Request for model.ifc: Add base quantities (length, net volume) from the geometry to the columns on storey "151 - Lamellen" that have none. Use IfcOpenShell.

First a look at what the model holds.

```python
import ifcopenshell
import ifcopenshell.util.element
import ifcopenshell.util.unit

model = ifcopenshell.open("model.ifc")
print(model.schema)
for unit_type in ("LENGTHUNIT", "AREAUNIT", "VOLUMEUNIT"):
    print(unit_type, ifcopenshell.util.unit.calculate_unit_scale(model, unit_type))
storey = next(s for s in model.by_type("IfcBuildingStorey") if s.Name == "151 - Lamellen")
columns = [e for e in ifcopenshell.util.element.get_decomposition(storey) if e.is_a("IfcColumn")]
for e in sorted(columns, key=lambda e: e.id()):
    print(e.id(), e.is_a(), e.Name, list(ifcopenshell.util.element.get_psets(e, qtos_only=True)), sep=" | ")
```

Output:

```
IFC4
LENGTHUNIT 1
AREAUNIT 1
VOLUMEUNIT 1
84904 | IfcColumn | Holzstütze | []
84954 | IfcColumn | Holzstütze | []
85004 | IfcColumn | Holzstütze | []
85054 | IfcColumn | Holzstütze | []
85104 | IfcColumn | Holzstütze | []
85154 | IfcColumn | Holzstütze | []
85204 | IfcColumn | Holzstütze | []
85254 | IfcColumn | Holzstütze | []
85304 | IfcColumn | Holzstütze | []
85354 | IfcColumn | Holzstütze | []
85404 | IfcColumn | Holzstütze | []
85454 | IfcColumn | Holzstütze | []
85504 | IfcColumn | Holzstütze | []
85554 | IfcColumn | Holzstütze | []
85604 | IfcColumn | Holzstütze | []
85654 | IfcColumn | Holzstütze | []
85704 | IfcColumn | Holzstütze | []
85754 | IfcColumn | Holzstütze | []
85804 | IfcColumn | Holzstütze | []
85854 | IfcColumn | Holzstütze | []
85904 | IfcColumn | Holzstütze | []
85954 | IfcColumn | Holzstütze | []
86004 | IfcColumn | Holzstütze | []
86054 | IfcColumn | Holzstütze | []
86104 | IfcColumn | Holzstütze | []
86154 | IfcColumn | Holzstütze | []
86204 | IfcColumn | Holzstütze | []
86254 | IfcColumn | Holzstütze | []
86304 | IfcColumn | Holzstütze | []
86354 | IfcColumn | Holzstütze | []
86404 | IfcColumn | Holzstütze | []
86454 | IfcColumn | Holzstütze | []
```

```python
import ifcopenshell
import ifcopenshell.api.pset
import ifcopenshell.geom
import ifcopenshell.util.element
import ifcopenshell.util.shape
import ifcopenshell.util.unit

model = ifcopenshell.open("model.ifc")
unit_scale = ifcopenshell.util.unit.calculate_unit_scale(model)
volume_scale = ifcopenshell.util.unit.calculate_unit_scale(model, "VOLUMEUNIT")
settings = ifcopenshell.geom.settings()

storey = next(s for s in model.by_type("IfcBuildingStorey") if s.Name == "151 - Lamellen")
columns = [e for e in ifcopenshell.util.element.get_decomposition(storey) if e.is_a("IfcColumn")]

for e in sorted(columns, key=lambda e: e.id()):
    if ifcopenshell.util.element.get_psets(e, qtos_only=True, should_inherit=False):
        continue
    # Geometry comes back in metres, in the element's own axes.
    shape = ifcopenshell.geom.create_shape(settings, e)
    values = {
        "Length": ifcopenshell.util.shape.get_z(shape.geometry) / unit_scale,
        "NetVolume": ifcopenshell.util.shape.get_volume(shape.geometry) / volume_scale,
    }
    qto = ifcopenshell.api.pset.add_qto(model, product=e, name="Qto_ColumnBaseQuantities")
    ifcopenshell.api.pset.edit_qto(model, qto=qto, properties=values)
    print(e.id(), {k: round(v, 3) for k, v in values.items()})

model.write("model_updated.ifc")
```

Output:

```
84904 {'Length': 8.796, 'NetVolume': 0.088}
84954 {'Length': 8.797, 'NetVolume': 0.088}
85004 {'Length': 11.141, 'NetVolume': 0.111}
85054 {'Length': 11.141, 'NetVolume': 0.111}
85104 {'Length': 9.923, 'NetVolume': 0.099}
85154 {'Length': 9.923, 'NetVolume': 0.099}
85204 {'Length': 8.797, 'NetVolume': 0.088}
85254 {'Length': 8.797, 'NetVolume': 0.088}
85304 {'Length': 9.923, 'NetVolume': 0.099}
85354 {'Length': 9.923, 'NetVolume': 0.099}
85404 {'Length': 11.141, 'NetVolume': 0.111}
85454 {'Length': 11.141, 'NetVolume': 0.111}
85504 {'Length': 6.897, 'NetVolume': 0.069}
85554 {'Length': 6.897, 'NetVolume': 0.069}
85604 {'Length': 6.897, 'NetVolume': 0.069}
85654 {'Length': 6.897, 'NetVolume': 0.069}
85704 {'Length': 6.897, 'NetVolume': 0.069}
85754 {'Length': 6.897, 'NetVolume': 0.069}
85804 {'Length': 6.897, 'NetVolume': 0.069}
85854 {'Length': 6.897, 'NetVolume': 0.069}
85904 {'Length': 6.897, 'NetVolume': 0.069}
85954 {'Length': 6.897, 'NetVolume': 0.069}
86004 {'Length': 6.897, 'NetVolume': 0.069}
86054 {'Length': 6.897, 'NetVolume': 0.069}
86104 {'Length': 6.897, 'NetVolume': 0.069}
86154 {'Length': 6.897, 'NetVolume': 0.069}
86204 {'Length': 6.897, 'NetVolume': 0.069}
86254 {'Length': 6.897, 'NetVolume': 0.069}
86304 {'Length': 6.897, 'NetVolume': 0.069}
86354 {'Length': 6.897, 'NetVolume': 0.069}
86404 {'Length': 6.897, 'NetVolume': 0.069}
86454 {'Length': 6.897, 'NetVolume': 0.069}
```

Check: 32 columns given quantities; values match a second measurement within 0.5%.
